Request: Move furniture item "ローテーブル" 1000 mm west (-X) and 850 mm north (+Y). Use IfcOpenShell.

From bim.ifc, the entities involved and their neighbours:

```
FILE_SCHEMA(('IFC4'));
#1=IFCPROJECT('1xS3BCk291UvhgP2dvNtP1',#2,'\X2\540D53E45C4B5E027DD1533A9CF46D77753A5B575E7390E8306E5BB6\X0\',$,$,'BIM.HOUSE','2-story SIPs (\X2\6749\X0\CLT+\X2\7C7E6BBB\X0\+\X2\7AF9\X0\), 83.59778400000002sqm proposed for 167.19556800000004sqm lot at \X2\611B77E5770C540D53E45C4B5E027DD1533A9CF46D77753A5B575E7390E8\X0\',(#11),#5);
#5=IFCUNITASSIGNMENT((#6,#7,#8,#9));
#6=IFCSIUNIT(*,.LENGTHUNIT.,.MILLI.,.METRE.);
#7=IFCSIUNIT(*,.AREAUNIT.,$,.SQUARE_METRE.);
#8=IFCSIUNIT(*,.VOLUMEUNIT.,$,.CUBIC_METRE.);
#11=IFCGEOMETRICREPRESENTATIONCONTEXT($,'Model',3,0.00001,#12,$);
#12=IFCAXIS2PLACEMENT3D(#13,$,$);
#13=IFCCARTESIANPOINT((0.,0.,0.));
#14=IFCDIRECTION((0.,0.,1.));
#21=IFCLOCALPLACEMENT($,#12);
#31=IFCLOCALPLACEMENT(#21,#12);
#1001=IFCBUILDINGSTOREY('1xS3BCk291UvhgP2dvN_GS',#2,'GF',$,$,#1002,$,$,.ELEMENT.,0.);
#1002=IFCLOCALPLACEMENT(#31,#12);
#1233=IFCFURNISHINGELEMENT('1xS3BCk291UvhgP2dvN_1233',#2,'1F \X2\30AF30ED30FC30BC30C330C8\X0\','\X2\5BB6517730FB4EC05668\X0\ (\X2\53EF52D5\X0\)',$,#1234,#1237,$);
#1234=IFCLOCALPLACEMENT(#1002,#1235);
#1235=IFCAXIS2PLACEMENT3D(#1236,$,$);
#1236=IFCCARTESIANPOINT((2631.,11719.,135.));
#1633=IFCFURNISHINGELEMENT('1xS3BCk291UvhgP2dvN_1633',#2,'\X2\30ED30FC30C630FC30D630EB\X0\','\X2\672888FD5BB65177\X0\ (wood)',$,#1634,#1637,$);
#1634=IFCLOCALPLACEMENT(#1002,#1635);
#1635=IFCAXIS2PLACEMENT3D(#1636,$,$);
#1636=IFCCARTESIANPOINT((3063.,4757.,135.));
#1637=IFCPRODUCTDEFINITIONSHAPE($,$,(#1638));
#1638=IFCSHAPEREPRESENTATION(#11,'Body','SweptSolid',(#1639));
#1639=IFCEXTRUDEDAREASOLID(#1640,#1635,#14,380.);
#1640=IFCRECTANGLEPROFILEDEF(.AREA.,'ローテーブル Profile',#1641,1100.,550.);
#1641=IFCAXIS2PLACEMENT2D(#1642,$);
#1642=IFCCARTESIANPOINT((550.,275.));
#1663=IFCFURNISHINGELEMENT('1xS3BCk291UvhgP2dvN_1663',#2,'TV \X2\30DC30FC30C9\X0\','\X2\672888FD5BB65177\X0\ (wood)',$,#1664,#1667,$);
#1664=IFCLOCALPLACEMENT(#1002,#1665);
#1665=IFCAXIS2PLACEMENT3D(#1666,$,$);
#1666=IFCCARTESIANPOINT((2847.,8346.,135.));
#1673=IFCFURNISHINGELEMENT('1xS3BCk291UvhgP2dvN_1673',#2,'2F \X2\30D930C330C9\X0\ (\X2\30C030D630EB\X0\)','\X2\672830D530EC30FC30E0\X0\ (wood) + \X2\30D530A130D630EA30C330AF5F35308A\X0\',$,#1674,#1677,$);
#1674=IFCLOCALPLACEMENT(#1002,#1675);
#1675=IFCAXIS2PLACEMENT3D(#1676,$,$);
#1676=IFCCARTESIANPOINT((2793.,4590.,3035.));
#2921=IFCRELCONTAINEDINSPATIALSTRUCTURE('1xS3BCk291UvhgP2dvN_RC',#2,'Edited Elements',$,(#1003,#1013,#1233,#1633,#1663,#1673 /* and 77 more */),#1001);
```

```python
import ifcopenshell
import ifcopenshell.api.geometry
import ifcopenshell.util.placement

model = ifcopenshell.open("bim.ifc")

item = model.by_guid("1xS3BCk291UvhgP2dvN_1633")
matrix = ifcopenshell.util.placement.get_local_placement(item.ObjectPlacement)
matrix[0, 3] -= 1000.0
matrix[1, 3] += 850.0
ifcopenshell.api.geometry.edit_object_placement(model, product=item, matrix=matrix, is_si=False)

print(ifcopenshell.util.placement.get_local_placement(item.ObjectPlacement).round(3) + 0.0)

model.write("bim_rev.ifc")
```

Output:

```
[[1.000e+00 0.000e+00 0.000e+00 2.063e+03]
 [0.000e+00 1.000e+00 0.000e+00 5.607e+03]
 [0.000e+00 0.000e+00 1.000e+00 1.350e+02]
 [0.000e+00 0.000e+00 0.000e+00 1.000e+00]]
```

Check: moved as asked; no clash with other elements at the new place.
